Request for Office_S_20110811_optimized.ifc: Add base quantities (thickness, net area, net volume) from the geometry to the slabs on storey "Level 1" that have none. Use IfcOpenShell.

First a look at what the model holds.

```python
import ifcopenshell
import ifcopenshell.util.element
import ifcopenshell.util.unit

model = ifcopenshell.open("Office_S_20110811_optimized.ifc")
print(model.schema)
for unit_type in ("LENGTHUNIT", "AREAUNIT", "VOLUMEUNIT"):
    print(unit_type, ifcopenshell.util.unit.calculate_unit_scale(model, unit_type))
storey = next(s for s in model.by_type("IfcBuildingStorey") if s.Name == "Level 1")
slabs = [e for e in ifcopenshell.util.element.get_decomposition(storey) if e.is_a("IfcSlab")]
for e in sorted(slabs, key=lambda e: e.id()):
    print(e.id(), e.is_a(), e.Name, list(ifcopenshell.util.element.get_psets(e, qtos_only=True)), sep=" | ")
```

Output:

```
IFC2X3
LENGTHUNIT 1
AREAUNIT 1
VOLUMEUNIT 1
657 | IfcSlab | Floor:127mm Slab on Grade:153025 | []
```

```python
import ifcopenshell
import ifcopenshell.api.pset
import ifcopenshell.geom
import ifcopenshell.util.element
import ifcopenshell.util.shape
import ifcopenshell.util.unit

model = ifcopenshell.open("Office_S_20110811_optimized.ifc")
unit_scale = ifcopenshell.util.unit.calculate_unit_scale(model)
area_scale = ifcopenshell.util.unit.calculate_unit_scale(model, "AREAUNIT")
volume_scale = ifcopenshell.util.unit.calculate_unit_scale(model, "VOLUMEUNIT")
settings = ifcopenshell.geom.settings()

storey = next(s for s in model.by_type("IfcBuildingStorey") if s.Name == "Level 1")
slabs = [e for e in ifcopenshell.util.element.get_decomposition(storey) if e.is_a("IfcSlab")]

for e in sorted(slabs, key=lambda e: e.id()):
    if ifcopenshell.util.element.get_psets(e, qtos_only=True, should_inherit=False):
        continue
    # Geometry comes back in metres, in the element's own axes.
    shape = ifcopenshell.geom.create_shape(settings, e)
    values = {
        "Width": ifcopenshell.util.shape.get_z(shape.geometry) / unit_scale,
        "NetArea": ifcopenshell.util.shape.get_footprint_area(shape.geometry) / area_scale,
        "NetVolume": ifcopenshell.util.shape.get_volume(shape.geometry) / volume_scale,
    }
    qto = ifcopenshell.api.pset.add_qto(model, product=e, name="BaseQuantities")
    ifcopenshell.api.pset.edit_qto(model, qto=qto, properties=values)
    print(e.id(), {k: round(v, 3) for k, v in values.items()})

model.write("Office_S_20110811_optimized_updated.ifc")
```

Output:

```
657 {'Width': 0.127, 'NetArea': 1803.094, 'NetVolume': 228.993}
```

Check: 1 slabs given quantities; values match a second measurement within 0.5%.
